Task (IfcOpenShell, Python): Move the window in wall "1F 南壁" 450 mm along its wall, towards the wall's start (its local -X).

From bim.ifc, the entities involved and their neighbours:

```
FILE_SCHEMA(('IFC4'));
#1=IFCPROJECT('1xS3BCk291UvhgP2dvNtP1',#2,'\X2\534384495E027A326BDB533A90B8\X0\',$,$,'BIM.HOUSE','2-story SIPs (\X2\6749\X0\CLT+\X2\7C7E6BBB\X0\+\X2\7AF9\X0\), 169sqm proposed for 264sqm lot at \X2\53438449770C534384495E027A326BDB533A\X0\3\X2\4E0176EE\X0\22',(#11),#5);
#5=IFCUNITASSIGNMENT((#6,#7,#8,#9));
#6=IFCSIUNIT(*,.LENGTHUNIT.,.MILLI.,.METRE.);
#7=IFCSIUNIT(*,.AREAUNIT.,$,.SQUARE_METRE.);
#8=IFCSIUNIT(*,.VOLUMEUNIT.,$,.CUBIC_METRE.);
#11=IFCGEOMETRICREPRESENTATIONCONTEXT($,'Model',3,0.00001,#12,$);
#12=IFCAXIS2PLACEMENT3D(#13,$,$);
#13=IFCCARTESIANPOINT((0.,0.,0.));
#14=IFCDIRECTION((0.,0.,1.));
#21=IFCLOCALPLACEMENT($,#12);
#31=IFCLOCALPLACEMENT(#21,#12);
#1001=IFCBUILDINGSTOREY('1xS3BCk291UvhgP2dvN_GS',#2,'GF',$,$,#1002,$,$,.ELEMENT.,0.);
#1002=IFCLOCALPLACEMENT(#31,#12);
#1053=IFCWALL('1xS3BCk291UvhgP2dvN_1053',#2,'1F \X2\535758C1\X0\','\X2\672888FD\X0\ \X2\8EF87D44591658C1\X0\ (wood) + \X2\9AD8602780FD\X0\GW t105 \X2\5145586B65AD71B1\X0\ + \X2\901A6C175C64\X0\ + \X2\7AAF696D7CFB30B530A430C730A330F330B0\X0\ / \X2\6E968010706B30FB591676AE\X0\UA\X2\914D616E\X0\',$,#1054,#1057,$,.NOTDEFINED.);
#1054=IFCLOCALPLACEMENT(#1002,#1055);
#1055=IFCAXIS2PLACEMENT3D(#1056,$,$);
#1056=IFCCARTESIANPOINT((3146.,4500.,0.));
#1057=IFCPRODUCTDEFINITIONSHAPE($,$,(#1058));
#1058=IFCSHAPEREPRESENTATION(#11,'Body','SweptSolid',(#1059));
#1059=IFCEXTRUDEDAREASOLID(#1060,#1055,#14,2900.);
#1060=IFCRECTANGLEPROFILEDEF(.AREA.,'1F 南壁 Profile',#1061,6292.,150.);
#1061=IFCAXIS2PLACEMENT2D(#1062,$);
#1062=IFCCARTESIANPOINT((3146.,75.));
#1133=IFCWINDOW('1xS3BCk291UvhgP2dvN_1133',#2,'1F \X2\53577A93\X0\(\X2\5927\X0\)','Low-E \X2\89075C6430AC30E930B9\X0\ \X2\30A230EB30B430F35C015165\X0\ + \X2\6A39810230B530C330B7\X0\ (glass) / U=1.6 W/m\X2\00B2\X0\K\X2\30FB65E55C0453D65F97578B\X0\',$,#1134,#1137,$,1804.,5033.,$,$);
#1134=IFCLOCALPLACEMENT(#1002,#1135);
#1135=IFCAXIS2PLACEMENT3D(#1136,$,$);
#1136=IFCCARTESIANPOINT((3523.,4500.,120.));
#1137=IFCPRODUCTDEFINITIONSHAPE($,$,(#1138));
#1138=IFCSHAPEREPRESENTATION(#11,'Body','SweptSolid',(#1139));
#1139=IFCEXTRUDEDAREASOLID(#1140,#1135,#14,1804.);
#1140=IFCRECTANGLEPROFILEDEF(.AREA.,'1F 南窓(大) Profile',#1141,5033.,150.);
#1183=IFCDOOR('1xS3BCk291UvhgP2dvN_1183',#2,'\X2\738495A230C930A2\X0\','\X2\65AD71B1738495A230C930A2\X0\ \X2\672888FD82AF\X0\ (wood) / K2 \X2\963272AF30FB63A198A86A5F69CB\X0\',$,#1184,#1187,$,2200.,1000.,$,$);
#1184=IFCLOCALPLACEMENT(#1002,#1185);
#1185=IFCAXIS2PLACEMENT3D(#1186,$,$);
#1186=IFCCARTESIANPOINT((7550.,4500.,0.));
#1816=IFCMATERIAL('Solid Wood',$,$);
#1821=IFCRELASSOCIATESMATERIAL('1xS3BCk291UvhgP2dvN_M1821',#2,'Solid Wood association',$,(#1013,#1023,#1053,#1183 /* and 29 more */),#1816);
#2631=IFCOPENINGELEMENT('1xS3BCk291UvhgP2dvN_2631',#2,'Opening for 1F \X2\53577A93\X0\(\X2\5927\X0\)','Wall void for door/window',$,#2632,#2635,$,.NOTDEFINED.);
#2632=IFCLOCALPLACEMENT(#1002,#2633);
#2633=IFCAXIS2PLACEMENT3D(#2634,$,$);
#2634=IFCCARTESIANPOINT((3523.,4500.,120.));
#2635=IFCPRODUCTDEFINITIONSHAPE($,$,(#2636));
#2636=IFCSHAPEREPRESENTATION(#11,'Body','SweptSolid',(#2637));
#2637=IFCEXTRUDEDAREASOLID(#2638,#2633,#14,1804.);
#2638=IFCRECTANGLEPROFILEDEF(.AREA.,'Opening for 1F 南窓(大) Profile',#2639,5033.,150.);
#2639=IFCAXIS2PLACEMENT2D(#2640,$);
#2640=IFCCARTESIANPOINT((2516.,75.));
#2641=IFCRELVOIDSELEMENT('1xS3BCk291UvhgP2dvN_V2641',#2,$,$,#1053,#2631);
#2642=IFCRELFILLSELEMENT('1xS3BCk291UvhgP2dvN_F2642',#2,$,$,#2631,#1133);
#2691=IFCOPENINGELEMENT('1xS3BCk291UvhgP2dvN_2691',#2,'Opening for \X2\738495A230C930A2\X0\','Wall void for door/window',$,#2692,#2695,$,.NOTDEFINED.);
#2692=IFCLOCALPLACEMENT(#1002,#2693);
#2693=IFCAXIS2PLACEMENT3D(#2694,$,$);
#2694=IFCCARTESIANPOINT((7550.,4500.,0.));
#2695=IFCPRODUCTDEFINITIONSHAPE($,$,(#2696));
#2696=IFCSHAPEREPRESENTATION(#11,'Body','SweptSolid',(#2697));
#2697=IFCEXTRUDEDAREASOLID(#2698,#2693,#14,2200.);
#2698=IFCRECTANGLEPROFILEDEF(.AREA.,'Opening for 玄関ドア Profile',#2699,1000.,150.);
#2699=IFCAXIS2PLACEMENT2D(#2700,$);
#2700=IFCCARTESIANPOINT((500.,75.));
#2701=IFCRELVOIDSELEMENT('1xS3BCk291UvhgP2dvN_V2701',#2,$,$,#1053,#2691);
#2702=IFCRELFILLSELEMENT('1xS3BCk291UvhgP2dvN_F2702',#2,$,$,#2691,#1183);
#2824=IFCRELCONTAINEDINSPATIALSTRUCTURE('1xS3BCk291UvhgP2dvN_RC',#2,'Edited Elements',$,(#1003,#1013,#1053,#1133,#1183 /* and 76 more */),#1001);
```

```python
import ifcopenshell
import ifcopenshell.api.geometry
import ifcopenshell.util.placement

model = ifcopenshell.open("bim.ifc")

window = model.by_id(1133)
opening = window.FillsVoids[0].RelatingOpeningElement
wall = opening.VoidsElements[0].RelatingBuildingElement

wall_matrix = ifcopenshell.util.placement.get_local_placement(wall.ObjectPlacement)
shift = wall_matrix[:3, 0] * -450.0
before = ifcopenshell.util.placement.get_local_placement(window.ObjectPlacement)[:3, 3].copy()

# The window is not placed relative to its opening, so move both.
for product in (opening, window):
    matrix = ifcopenshell.util.placement.get_local_placement(product.ObjectPlacement)
    matrix[:3, 3] += shift
    ifcopenshell.api.geometry.edit_object_placement(model, product=product, matrix=matrix, is_si=False)

after = ifcopenshell.util.placement.get_local_placement(window.ObjectPlacement)[:3, 3]
print("window moved by", (after - before).round(3) + 0.0)

model.write("bim-out.ifc")
```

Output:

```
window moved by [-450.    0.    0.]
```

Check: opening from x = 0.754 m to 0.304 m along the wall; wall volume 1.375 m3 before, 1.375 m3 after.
